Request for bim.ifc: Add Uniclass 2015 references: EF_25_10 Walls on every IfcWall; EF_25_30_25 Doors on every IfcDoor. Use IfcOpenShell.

First a look at what the model holds.

```python
import ifcopenshell

model = ifcopenshell.open("bim.ifc")
print(model.schema)
print("classifications:", [c.Name for c in model.by_type("IfcClassification")])
for ifc_class in ("IfcDoor", "IfcRoof", "IfcStair", "IfcWall", "IfcWindow"):
    print(ifc_class, len(model.by_type(ifc_class)))
```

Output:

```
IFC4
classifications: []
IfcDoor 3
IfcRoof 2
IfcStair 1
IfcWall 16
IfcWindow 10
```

```python
import ifcopenshell
import ifcopenshell.api.classification

model = ifcopenshell.open("bim.ifc")

system = ifcopenshell.api.classification.add_classification(model, classification="Uniclass 2015")

codes = {
    "IfcWall": ("EF_25_10", "Walls"),
    "IfcDoor": ("EF_25_30_25", "Doors"),
}
for ifc_class, (code, name) in codes.items():
    products = model.by_type(ifc_class)
    ifcopenshell.api.classification.add_reference(
        model, products=products, classification=system, identification=code, name=name
    )
    print(code, len(products))

model.write("bim_rev.ifc")
```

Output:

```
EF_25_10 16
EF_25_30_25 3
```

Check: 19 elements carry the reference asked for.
